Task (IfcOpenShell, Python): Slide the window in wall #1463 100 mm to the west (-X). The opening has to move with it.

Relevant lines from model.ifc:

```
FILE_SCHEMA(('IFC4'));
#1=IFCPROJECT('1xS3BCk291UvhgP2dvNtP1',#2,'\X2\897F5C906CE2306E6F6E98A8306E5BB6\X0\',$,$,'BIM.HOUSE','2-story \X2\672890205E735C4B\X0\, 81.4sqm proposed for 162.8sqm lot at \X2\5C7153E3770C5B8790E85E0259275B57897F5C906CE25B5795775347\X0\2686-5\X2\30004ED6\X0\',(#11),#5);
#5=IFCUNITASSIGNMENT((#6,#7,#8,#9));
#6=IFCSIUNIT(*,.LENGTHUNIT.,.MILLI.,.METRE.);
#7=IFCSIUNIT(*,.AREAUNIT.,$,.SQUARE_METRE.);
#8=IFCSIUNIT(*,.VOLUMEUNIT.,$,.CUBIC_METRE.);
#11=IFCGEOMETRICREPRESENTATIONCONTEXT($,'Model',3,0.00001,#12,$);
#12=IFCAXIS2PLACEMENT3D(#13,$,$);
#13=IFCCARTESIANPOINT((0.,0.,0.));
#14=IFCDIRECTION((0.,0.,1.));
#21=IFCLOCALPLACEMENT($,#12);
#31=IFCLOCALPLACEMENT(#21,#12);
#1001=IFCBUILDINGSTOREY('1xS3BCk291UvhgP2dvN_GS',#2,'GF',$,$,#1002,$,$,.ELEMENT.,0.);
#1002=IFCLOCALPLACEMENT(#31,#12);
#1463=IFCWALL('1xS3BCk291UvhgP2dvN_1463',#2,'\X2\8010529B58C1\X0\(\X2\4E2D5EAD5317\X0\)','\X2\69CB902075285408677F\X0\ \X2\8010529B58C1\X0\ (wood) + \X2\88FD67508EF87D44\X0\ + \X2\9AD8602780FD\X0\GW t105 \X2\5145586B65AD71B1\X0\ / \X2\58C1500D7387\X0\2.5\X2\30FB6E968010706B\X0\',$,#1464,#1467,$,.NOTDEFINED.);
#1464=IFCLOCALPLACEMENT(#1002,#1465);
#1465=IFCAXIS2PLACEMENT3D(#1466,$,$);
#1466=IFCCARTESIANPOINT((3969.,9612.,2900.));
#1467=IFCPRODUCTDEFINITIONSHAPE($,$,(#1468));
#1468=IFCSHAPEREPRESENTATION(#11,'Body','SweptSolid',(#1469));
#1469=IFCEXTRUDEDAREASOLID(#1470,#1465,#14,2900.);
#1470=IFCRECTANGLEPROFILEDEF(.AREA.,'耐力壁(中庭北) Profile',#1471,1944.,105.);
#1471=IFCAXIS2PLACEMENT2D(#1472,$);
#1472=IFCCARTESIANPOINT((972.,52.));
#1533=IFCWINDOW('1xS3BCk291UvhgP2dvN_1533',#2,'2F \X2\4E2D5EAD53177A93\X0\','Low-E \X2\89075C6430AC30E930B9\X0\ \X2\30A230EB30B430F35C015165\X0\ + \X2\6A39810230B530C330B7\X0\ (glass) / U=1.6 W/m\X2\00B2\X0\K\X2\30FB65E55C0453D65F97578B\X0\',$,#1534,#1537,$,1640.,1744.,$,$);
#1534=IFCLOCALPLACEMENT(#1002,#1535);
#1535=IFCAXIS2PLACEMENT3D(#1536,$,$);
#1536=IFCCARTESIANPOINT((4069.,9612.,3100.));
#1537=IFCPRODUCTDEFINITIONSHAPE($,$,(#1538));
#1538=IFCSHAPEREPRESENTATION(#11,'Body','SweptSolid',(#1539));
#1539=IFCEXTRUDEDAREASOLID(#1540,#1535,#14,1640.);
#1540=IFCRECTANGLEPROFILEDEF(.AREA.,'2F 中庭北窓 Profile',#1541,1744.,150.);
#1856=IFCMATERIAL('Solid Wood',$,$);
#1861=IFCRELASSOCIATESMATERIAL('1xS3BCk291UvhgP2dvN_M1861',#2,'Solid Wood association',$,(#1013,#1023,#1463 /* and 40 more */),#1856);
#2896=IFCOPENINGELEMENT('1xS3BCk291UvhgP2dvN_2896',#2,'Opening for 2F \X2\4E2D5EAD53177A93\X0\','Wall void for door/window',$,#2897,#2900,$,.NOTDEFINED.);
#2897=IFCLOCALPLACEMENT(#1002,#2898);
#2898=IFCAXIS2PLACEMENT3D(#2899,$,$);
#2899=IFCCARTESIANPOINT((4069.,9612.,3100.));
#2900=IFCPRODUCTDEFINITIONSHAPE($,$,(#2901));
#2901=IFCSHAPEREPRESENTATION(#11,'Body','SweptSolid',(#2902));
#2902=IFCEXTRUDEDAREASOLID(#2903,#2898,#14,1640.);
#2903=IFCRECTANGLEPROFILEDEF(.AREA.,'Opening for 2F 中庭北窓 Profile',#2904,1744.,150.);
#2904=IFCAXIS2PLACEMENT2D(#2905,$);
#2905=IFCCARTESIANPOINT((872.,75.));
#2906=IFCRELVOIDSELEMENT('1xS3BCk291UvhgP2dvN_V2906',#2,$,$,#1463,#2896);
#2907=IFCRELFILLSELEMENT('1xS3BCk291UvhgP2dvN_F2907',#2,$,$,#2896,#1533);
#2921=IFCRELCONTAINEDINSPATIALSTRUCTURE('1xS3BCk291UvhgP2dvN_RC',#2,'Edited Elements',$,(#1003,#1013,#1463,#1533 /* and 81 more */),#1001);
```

```python
import ifcopenshell
import ifcopenshell.api.geometry
import ifcopenshell.util.placement
import ifcopenshell.util.unit

model = ifcopenshell.open("model.ifc")
unit_scale = ifcopenshell.util.unit.calculate_unit_scale(model)

window = model.by_guid("1xS3BCk291UvhgP2dvN_1533")
opening = window.FillsVoids[0].RelatingOpeningElement
wall = opening.VoidsElements[0].RelatingBuildingElement

wall_matrix = ifcopenshell.util.placement.get_local_placement(wall.ObjectPlacement)
shift = wall_matrix[:3, 0] * -0.1 / unit_scale
before = ifcopenshell.util.placement.get_local_placement(window.ObjectPlacement)[:3, 3].copy()

# The window is not placed relative to its opening, so move both.
for product in (opening, window):
    matrix = ifcopenshell.util.placement.get_local_placement(product.ObjectPlacement)
    matrix[:3, 3] += shift
    ifcopenshell.api.geometry.edit_object_placement(model, product=product, matrix=matrix, is_si=False)

after = ifcopenshell.util.placement.get_local_placement(window.ObjectPlacement)[:3, 3]
print("window moved by", (after - before).round(3) + 0.0)

model.write("model_updated.ifc")
```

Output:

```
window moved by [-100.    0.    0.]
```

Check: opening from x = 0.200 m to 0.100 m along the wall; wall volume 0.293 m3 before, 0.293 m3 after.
